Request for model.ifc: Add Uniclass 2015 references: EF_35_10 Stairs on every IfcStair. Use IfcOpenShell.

First a look at what the model holds.

```python
import ifcopenshell

model = ifcopenshell.open("model.ifc")
print(model.schema)
print("classifications:", [c.Name for c in model.by_type("IfcClassification")])
for ifc_class in ("IfcDoor", "IfcRoof", "IfcStair", "IfcWall", "IfcWindow"):
    print(ifc_class, len(model.by_type(ifc_class)))
```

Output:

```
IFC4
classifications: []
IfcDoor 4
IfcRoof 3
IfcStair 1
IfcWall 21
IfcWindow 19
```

```python
import ifcopenshell
import ifcopenshell.api.classification

model = ifcopenshell.open("model.ifc")

system = ifcopenshell.api.classification.add_classification(model, classification="Uniclass 2015")

codes = {
    "IfcStair": ("EF_35_10", "Stairs"),
}
for ifc_class, (code, name) in codes.items():
    products = model.by_type(ifc_class)
    ifcopenshell.api.classification.add_reference(
        model, products=products, classification=system, identification=code, name=name
    )
    print(code, len(products))

model.write("model_updated.ifc")
```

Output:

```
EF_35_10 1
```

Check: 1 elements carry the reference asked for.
